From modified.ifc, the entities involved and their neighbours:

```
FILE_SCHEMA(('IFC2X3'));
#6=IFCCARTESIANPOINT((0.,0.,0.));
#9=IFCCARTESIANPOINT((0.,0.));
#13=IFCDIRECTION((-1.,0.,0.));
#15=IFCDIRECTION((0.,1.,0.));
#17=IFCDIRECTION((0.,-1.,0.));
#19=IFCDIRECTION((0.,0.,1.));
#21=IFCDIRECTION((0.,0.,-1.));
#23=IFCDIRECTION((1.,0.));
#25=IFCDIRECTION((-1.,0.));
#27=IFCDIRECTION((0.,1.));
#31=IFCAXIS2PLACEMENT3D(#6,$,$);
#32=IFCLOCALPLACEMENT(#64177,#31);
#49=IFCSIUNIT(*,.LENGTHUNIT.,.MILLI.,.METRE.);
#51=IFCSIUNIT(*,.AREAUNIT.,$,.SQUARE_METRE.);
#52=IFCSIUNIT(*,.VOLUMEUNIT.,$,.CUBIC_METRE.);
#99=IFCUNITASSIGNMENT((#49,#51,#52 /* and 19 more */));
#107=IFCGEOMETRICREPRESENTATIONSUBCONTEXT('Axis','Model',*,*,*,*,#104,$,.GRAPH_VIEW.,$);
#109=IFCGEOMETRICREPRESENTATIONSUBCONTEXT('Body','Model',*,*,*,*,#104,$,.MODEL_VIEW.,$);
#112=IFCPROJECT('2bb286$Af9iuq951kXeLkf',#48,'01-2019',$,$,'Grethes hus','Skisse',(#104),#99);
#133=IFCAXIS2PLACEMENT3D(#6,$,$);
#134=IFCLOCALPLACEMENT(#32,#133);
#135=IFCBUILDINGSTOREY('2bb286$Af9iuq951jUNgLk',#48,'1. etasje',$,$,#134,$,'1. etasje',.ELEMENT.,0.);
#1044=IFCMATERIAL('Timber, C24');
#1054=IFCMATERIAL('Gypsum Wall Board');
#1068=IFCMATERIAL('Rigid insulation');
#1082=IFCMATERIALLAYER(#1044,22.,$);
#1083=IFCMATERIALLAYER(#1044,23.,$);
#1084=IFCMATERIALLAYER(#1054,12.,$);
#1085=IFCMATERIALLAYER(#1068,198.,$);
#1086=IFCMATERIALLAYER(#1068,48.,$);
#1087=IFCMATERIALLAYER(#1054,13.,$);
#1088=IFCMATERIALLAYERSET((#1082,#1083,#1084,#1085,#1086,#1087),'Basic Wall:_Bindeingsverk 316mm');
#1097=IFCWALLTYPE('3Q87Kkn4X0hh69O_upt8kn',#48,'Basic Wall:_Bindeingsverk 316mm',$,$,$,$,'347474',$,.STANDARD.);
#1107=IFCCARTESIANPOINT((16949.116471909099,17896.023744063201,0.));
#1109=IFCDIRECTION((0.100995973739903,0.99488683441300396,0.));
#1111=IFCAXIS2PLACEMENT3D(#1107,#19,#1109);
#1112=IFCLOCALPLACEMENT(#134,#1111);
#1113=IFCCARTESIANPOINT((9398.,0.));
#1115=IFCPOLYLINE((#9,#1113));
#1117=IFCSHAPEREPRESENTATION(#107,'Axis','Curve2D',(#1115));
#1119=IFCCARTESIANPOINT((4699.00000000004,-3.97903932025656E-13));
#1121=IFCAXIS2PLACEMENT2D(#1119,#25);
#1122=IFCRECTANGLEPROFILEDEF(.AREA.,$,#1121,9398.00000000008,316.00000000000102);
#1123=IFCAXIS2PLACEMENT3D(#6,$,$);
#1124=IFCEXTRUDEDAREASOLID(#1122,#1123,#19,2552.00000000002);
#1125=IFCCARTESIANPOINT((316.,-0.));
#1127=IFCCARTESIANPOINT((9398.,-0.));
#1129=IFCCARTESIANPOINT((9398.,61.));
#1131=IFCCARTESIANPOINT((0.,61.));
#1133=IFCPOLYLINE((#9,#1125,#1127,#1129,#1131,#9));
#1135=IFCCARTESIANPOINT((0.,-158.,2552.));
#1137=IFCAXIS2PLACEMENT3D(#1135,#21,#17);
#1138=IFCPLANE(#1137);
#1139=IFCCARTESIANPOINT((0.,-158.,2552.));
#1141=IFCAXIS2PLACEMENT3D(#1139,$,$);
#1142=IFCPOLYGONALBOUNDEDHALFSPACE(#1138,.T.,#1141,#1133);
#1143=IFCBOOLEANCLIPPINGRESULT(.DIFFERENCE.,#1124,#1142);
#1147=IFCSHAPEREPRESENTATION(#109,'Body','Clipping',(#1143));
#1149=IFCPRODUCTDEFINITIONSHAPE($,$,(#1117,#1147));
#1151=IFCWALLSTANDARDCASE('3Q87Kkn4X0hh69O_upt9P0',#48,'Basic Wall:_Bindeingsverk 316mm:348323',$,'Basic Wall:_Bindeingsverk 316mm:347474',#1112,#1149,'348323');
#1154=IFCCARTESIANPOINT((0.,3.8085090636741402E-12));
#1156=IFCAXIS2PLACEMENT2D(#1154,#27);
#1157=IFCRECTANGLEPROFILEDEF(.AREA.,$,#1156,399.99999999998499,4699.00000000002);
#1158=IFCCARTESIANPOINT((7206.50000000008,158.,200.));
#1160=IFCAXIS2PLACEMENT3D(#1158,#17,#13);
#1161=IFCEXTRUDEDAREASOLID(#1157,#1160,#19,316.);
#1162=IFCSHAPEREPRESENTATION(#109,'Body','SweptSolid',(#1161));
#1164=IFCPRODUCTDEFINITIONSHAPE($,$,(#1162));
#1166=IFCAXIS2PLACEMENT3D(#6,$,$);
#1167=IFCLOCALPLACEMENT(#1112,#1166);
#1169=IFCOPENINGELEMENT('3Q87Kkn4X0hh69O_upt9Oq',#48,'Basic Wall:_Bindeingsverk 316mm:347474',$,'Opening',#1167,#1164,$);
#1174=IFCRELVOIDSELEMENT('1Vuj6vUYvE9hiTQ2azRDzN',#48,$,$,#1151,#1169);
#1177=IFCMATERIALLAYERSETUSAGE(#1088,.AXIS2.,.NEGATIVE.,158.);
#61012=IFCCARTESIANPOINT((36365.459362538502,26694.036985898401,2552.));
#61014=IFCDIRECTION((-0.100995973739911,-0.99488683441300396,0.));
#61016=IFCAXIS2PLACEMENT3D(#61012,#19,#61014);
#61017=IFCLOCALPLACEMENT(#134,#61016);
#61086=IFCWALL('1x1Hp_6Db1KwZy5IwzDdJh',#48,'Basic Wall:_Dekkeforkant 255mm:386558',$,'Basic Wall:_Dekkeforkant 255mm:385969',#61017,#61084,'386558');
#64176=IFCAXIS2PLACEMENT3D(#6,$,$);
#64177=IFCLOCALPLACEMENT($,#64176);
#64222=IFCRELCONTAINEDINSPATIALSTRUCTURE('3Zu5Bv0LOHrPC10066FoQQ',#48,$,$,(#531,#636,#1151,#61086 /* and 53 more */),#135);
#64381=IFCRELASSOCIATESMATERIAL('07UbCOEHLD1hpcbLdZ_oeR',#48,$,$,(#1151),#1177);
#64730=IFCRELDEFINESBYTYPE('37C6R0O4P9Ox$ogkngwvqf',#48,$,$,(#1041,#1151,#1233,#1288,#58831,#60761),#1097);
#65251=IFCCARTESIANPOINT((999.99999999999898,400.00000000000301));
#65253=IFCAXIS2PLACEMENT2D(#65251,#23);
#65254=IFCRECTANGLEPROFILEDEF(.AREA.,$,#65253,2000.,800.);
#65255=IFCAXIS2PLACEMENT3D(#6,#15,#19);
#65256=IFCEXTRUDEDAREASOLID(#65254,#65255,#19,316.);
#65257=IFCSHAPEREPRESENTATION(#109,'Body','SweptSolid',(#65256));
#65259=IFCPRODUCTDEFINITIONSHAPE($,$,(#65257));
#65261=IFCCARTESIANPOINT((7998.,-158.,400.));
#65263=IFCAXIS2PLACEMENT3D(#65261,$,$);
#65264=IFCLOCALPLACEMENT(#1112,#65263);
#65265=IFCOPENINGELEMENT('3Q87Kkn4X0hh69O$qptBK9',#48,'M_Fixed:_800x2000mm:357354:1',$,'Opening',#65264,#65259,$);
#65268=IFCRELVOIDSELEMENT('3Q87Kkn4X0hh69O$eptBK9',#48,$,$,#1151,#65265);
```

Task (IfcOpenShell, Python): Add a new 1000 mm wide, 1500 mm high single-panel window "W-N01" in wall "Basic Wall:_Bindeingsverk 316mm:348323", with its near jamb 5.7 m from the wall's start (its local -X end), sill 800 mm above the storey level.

```python
import numpy as np
import ifcopenshell
import ifcopenshell.api.feature
import ifcopenshell.api.geometry
import ifcopenshell.api.root
import ifcopenshell.api.spatial
import ifcopenshell.api.type
import ifcopenshell.geom
import ifcopenshell.util.element
import ifcopenshell.util.placement
import ifcopenshell.util.representation
import ifcopenshell.util.shape
import ifcopenshell.util.unit

model = ifcopenshell.open("modified.ifc")
unit_scale = ifcopenshell.util.unit.calculate_unit_scale(model)
settings = ifcopenshell.geom.settings()


def volume(element):
    """Net volume in cubic metres, openings subtracted."""
    shape = ifcopenshell.geom.create_shape(settings, element)
    return ifcopenshell.util.shape.get_volume(shape.geometry)


wall = model.by_guid("3Q87Kkn4X0hh69O_upt9P0")
storey = ifcopenshell.util.element.get_container(wall, ifc_class="IfcBuildingStorey")
context = ifcopenshell.util.representation.get_context(model, "Model", "Body", "MODEL_VIEW")
before = volume(wall)

width, height, from_end, sill = 1, 1.5, 5.7, 0.8  # metres

# The wall runs along its own X axis, and the end named is its -X end.
wall_shape = ifcopenshell.geom.create_shape(settings, wall)
x, y, z = ifcopenshell.util.shape.get_vertices(wall_shape.geometry).T
start = x.min() + from_end
face, thickness = float(y.min()), float(y.max() - y.min())
wall_matrix = ifcopenshell.util.placement.get_local_placement(wall.ObjectPlacement)
level = ifcopenshell.util.placement.get_local_placement(storey.ObjectPlacement)[2, 3]


def in_wall(x, y):
    """Placement at x, y metres in the wall's axes, at sill height."""
    matrix = wall_matrix.copy()
    matrix[:, 3] = wall_matrix @ np.array([x / unit_scale, y / unit_scale, 0.0, 1.0])
    matrix[2, 3] = level + sill / unit_scale
    return matrix


# Opening: a box that overshoots both wall faces by 50 mm.
opening = ifcopenshell.api.root.create_entity(model, ifc_class="IfcOpeningElement")
box = ifcopenshell.api.geometry.add_wall_representation(
    model, context=context, length=width, height=height, thickness=thickness + 0.1
)
ifcopenshell.api.geometry.assign_representation(model, product=opening, representation=box)
ifcopenshell.api.geometry.edit_object_placement(model, product=opening, matrix=in_wall(start, face - 0.05), is_si=False)
ifcopenshell.api.feature.add_feature(model, feature=opening, element=wall)

window = ifcopenshell.api.root.create_entity(model, ifc_class="IfcWindow", name="W-N01")
window.OverallWidth, window.OverallHeight = width / unit_scale, height / unit_scale
body = ifcopenshell.api.geometry.add_window_representation(
    model,
    context=context,
    overall_width=window.OverallWidth,
    overall_height=window.OverallHeight,
    partition_type="SINGLE_PANEL",
)
ifcopenshell.api.geometry.assign_representation(model, product=window, representation=body)
ifcopenshell.api.spatial.assign_container(model, products=[window], relating_structure=storey)
fills = ifcopenshell.api.feature.add_filling(model, opening=opening, element=window)
fills.OwnerHistory = window.OwnerHistory  # required in IFC2X3

# IFC2X3 keeps the operation on the window style.
style = ifcopenshell.api.root.create_entity(model, ifc_class="IfcWindowStyle", name="W-N01")
style.OperationType, style.ConstructionType = "SINGLE_PANEL", "NOTDEFINED"
style.ParameterTakesPrecedence = style.Sizeable = False
ifcopenshell.api.type.assign_type(model, related_objects=[window], relating_type=style)

# Centre the window in the wall's thickness.
ifcopenshell.api.geometry.edit_object_placement(model, product=window, matrix=in_wall(start, face), is_si=False)
window_shape = ifcopenshell.geom.create_shape(settings, window)
depth = ifcopenshell.util.shape.get_vertices(window_shape.geometry)[:, 1]
offset = face + thickness / 2 - (depth.min() + depth.max()) / 2
ifcopenshell.api.geometry.edit_object_placement(model, product=window, matrix=in_wall(start, offset), is_si=False)

after = volume(wall)

print(f"wall volume {before:.3f} -> {after:.3f} m3")

model.write("modified_rev.ifc")
```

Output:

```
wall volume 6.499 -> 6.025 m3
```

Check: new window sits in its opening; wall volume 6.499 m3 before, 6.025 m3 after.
